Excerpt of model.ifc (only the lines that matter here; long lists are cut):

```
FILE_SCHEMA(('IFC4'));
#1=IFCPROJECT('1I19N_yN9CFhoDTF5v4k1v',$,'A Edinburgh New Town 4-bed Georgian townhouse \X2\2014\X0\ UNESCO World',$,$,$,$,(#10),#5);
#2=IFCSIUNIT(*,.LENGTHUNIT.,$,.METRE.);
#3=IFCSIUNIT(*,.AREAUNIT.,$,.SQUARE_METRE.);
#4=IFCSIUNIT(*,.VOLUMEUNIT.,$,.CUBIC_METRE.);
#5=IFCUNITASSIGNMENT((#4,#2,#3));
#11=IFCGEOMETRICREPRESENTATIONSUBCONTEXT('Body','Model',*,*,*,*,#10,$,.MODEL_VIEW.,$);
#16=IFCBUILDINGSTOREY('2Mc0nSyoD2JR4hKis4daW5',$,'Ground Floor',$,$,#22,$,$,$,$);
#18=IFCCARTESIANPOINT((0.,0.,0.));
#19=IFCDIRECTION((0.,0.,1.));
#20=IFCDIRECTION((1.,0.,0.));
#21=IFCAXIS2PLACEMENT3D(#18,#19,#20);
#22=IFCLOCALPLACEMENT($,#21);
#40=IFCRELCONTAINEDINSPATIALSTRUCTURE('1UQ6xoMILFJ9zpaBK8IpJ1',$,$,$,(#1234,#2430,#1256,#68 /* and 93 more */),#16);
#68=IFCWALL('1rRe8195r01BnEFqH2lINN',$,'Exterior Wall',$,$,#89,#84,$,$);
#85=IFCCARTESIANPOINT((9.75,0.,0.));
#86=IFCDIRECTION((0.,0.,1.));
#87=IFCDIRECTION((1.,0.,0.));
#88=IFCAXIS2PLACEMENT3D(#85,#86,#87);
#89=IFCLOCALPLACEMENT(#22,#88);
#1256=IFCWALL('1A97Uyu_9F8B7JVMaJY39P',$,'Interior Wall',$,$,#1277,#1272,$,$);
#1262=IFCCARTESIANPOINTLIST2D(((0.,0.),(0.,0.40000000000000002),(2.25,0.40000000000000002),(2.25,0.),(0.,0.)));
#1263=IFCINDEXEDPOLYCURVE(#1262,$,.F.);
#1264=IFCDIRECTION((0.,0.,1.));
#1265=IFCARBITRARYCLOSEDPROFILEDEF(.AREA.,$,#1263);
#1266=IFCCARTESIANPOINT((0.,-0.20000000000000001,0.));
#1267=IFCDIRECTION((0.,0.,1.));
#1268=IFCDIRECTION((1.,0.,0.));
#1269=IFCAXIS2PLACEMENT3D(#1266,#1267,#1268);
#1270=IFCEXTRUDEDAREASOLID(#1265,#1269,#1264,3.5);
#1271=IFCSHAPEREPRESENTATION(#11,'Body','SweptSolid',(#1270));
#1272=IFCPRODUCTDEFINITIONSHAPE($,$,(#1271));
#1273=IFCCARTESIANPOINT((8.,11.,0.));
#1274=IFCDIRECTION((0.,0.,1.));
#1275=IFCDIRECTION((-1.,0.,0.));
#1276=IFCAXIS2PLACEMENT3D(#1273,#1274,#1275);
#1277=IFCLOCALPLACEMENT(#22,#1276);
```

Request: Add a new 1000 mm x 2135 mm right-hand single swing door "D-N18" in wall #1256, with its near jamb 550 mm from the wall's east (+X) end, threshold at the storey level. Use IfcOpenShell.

```python
import numpy as np
import ifcopenshell
import ifcopenshell.api.feature
import ifcopenshell.api.geometry
import ifcopenshell.api.root
import ifcopenshell.api.spatial
import ifcopenshell.geom
import ifcopenshell.util.element
import ifcopenshell.util.placement
import ifcopenshell.util.representation
import ifcopenshell.util.shape
import ifcopenshell.util.unit

model = ifcopenshell.open("model.ifc")
unit_scale = ifcopenshell.util.unit.calculate_unit_scale(model)
settings = ifcopenshell.geom.settings()


def volume(element):
    """Net volume in cubic metres, openings subtracted."""
    shape = ifcopenshell.geom.create_shape(settings, element)
    return ifcopenshell.util.shape.get_volume(shape.geometry)


wall = model.by_guid("1A97Uyu_9F8B7JVMaJY39P")
storey = ifcopenshell.util.element.get_container(wall, ifc_class="IfcBuildingStorey")
context = ifcopenshell.util.representation.get_context(model, "Model", "Body", "MODEL_VIEW")
before = volume(wall)

width, height, from_end, sill = 1, 2.135, 0.55, 0.0  # metres

# The wall runs along its own X axis, and the end named is its -X end.
wall_shape = ifcopenshell.geom.create_shape(settings, wall)
x, y, z = ifcopenshell.util.shape.get_vertices(wall_shape.geometry).T
start = x.min() + from_end
face, thickness = float(y.min()), float(y.max() - y.min())
wall_matrix = ifcopenshell.util.placement.get_local_placement(wall.ObjectPlacement)
level = ifcopenshell.util.placement.get_local_placement(storey.ObjectPlacement)[2, 3]


def in_wall(x, y):
    """Placement at x, y metres in the wall's axes, at sill height."""
    matrix = wall_matrix.copy()
    matrix[:, 3] = wall_matrix @ np.array([x / unit_scale, y / unit_scale, 0.0, 1.0])
    matrix[2, 3] = level + sill / unit_scale
    return matrix


# Opening: a box that overshoots both wall faces by 50 mm.
opening = ifcopenshell.api.root.create_entity(model, ifc_class="IfcOpeningElement", predefined_type="OPENING")
box = ifcopenshell.api.geometry.add_wall_representation(
    model, context=context, length=width, height=height, thickness=thickness + 0.1
)
ifcopenshell.api.geometry.assign_representation(model, product=opening, representation=box)
ifcopenshell.api.geometry.edit_object_placement(model, product=opening, matrix=in_wall(start, face - 0.05), is_si=False)
ifcopenshell.api.feature.add_feature(model, feature=opening, element=wall)

door = ifcopenshell.api.root.create_entity(model, ifc_class="IfcDoor", name="D-N18", predefined_type="DOOR")
door.OverallWidth, door.OverallHeight = width / unit_scale, height / unit_scale
door.OperationType = "SINGLE_SWING_RIGHT"
body = ifcopenshell.api.geometry.add_door_representation(
    model,
    context=context,
    overall_width=door.OverallWidth,
    overall_height=door.OverallHeight,
    operation_type="SINGLE_SWING_RIGHT",
    lining_properties={"LiningDepth": thickness / unit_scale, "ThresholdDepth": thickness / unit_scale},
)
ifcopenshell.api.geometry.assign_representation(model, product=door, representation=body)
ifcopenshell.api.spatial.assign_container(model, products=[door], relating_structure=storey)
ifcopenshell.api.feature.add_filling(model, opening=opening, element=door)

# The lining spans the wall, so the door starts at the wall face.
ifcopenshell.api.geometry.edit_object_placement(model, product=door, matrix=in_wall(start, face), is_si=False)

after = volume(wall)

print(f"wall volume {before:.3f} -> {after:.3f} m3")

model.write("model_rev.ifc")
```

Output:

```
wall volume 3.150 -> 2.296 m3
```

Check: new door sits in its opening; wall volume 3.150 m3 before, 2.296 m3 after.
